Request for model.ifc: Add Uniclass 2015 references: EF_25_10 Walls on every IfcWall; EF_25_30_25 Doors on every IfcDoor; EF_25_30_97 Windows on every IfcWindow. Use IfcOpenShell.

First a look at what the model holds.

```python
import ifcopenshell

model = ifcopenshell.open("model.ifc")
print(model.schema)
print("classifications:", [c.Name for c in model.by_type("IfcClassification")])
for ifc_class in ("IfcDoor", "IfcRoof", "IfcStair", "IfcWall", "IfcWindow"):
    print(ifc_class, len(model.by_type(ifc_class)))
```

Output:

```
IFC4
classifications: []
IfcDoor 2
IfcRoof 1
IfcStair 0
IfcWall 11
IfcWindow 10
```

```python
import ifcopenshell
import ifcopenshell.api.classification

model = ifcopenshell.open("model.ifc")

system = ifcopenshell.api.classification.add_classification(model, classification="Uniclass 2015")

codes = {
    "IfcWall": ("EF_25_10", "Walls"),
    "IfcDoor": ("EF_25_30_25", "Doors"),
    "IfcWindow": ("EF_25_30_97", "Windows"),
}
for ifc_class, (code, name) in codes.items():
    products = model.by_type(ifc_class)
    ifcopenshell.api.classification.add_reference(
        model, products=products, classification=system, identification=code, name=name
    )
    print(code, len(products))

model.write("model-out.ifc")
```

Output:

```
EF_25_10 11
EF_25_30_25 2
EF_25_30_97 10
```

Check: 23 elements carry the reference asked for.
